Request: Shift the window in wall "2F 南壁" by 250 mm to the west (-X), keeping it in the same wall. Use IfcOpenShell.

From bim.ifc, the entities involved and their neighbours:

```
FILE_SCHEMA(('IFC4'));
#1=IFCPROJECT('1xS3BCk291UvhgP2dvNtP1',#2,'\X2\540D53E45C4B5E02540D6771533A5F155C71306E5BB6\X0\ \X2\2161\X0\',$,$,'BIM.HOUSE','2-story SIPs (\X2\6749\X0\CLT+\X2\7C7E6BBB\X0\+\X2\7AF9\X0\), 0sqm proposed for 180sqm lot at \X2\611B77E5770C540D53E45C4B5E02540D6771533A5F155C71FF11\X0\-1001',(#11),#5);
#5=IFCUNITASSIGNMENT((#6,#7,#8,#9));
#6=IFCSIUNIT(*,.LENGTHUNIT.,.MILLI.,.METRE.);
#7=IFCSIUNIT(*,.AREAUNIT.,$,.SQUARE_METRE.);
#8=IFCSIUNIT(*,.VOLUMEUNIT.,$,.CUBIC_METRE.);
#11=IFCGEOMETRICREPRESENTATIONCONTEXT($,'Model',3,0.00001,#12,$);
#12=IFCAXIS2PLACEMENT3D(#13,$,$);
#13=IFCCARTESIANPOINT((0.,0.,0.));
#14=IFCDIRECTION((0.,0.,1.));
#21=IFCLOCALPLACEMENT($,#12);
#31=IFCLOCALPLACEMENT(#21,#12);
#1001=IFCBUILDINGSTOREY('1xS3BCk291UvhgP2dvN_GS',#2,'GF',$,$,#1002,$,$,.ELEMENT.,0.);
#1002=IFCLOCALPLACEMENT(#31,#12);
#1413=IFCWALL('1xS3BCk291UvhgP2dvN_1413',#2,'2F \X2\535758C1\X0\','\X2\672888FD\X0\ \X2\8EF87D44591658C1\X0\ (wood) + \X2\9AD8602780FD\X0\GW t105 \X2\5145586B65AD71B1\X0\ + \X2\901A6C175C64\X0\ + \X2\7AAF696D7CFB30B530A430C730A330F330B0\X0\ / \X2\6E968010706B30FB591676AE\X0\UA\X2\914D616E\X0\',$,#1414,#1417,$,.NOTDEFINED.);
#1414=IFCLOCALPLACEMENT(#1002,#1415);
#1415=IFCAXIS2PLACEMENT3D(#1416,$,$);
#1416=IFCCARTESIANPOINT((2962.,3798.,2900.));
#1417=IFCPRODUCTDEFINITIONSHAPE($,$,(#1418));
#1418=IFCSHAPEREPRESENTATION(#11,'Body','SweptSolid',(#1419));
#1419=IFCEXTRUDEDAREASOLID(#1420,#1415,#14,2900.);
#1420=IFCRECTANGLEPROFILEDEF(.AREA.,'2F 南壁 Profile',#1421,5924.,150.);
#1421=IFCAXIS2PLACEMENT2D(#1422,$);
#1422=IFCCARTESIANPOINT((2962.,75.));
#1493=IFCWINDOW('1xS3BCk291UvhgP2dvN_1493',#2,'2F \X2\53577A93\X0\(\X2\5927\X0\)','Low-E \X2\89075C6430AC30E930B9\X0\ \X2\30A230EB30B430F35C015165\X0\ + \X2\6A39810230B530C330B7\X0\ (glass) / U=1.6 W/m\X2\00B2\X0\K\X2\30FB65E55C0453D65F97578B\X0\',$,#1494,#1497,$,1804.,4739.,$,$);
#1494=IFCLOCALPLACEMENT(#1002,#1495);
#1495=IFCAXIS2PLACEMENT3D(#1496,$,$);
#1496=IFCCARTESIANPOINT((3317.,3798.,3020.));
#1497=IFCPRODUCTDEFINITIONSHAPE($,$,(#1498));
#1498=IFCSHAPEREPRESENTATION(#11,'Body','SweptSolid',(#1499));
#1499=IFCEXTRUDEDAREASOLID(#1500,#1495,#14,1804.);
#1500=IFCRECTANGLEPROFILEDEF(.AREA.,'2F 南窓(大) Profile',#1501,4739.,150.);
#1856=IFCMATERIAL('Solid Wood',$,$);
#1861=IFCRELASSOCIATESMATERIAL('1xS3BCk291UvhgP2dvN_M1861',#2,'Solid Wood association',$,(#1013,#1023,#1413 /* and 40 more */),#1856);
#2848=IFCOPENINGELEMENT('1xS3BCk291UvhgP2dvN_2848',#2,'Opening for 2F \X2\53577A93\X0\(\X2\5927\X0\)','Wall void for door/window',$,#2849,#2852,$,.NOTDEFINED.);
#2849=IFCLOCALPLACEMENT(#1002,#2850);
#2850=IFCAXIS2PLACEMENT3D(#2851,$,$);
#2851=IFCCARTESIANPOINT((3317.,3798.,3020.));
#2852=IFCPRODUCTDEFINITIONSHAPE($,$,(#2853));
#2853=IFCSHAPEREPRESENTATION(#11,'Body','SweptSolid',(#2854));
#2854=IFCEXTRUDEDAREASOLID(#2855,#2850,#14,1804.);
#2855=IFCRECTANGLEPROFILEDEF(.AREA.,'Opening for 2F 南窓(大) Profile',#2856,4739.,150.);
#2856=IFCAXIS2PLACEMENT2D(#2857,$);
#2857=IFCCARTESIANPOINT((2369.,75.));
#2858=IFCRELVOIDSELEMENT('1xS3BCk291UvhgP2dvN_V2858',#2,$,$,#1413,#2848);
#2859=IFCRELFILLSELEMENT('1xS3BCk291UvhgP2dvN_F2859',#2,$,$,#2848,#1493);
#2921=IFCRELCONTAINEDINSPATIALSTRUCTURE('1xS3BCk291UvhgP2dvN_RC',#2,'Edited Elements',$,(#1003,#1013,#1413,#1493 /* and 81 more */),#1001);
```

```python
import ifcopenshell
import ifcopenshell.api.geometry
import ifcopenshell.util.placement
import ifcopenshell.util.unit

model = ifcopenshell.open("bim.ifc")
unit_scale = ifcopenshell.util.unit.calculate_unit_scale(model)

window = model.by_guid("1xS3BCk291UvhgP2dvN_1493")
opening = window.FillsVoids[0].RelatingOpeningElement
wall = opening.VoidsElements[0].RelatingBuildingElement

wall_matrix = ifcopenshell.util.placement.get_local_placement(wall.ObjectPlacement)
shift = wall_matrix[:3, 0] * -0.25 / unit_scale
before = ifcopenshell.util.placement.get_local_placement(window.ObjectPlacement)[:3, 3].copy()

# The window is not placed relative to its opening, so move both.
for product in (opening, window):
    matrix = ifcopenshell.util.placement.get_local_placement(product.ObjectPlacement)
    matrix[:3, 3] += shift
    ifcopenshell.api.geometry.edit_object_placement(model, product=product, matrix=matrix, is_si=False)

after = ifcopenshell.util.placement.get_local_placement(window.ObjectPlacement)[:3, 3]
print("window moved by", (after - before).round(3) + 0.0)

model.write("bim_edited.ifc")
```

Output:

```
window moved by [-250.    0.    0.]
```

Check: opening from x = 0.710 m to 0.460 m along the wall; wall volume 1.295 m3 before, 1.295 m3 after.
